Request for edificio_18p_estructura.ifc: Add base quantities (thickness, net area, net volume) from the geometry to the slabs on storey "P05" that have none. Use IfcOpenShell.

First a look at what the model holds.

```python
import ifcopenshell
import ifcopenshell.util.element
import ifcopenshell.util.unit

model = ifcopenshell.open("edificio_18p_estructura.ifc")
print(model.schema)
for unit_type in ("LENGTHUNIT", "AREAUNIT", "VOLUMEUNIT"):
    print(unit_type, ifcopenshell.util.unit.calculate_unit_scale(model, unit_type))
storey = next(s for s in model.by_type("IfcBuildingStorey") if s.Name == "P05")
slabs = [e for e in ifcopenshell.util.element.get_decomposition(storey) if e.is_a("IfcSlab")]
for e in sorted(slabs, key=lambda e: e.id()):
    print(e.id(), e.is_a(), e.Name, list(ifcopenshell.util.element.get_psets(e, qtos_only=True)), sep=" | ")
```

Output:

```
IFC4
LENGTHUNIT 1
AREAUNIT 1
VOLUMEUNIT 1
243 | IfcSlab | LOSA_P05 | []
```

```python
import ifcopenshell
import ifcopenshell.api.pset
import ifcopenshell.geom
import ifcopenshell.util.element
import ifcopenshell.util.shape
import ifcopenshell.util.unit

model = ifcopenshell.open("edificio_18p_estructura.ifc")
unit_scale = ifcopenshell.util.unit.calculate_unit_scale(model)
area_scale = ifcopenshell.util.unit.calculate_unit_scale(model, "AREAUNIT")
volume_scale = ifcopenshell.util.unit.calculate_unit_scale(model, "VOLUMEUNIT")
settings = ifcopenshell.geom.settings()

storey = next(s for s in model.by_type("IfcBuildingStorey") if s.Name == "P05")
slabs = [e for e in ifcopenshell.util.element.get_decomposition(storey) if e.is_a("IfcSlab")]

for e in sorted(slabs, key=lambda e: e.id()):
    if ifcopenshell.util.element.get_psets(e, qtos_only=True, should_inherit=False):
        continue
    # Geometry comes back in metres, in the element's own axes.
    shape = ifcopenshell.geom.create_shape(settings, e)
    values = {
        "Width": ifcopenshell.util.shape.get_z(shape.geometry) / unit_scale,
        "NetArea": ifcopenshell.util.shape.get_footprint_area(shape.geometry) / area_scale,
        "NetVolume": ifcopenshell.util.shape.get_volume(shape.geometry) / volume_scale,
    }
    qto = ifcopenshell.api.pset.add_qto(model, product=e, name="Qto_SlabBaseQuantities")
    ifcopenshell.api.pset.edit_qto(model, qto=qto, properties=values)
    print(e.id(), {k: round(v, 3) for k, v in values.items()})

model.write("edificio_18p_estructura_edited.ifc")
```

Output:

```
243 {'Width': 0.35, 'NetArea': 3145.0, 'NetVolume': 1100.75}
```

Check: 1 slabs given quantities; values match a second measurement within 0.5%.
